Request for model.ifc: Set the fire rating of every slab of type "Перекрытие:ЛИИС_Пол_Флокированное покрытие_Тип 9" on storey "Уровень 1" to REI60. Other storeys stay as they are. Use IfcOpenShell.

First a look at what the model holds.

```python
import ifcopenshell
import ifcopenshell.util.element

model = ifcopenshell.open("model.ifc")
print(model.schema)
storey = next(s for s in model.by_type("IfcBuildingStorey") if s.Name == "Уровень 1")
slabs = [e for e in ifcopenshell.util.element.get_decomposition(storey) if e.is_a("IfcSlab")]
seen = {}
for e in slabs:
    element_type = ifcopenshell.util.element.get_type(e)
    key = (element_type.Name if element_type != e and element_type else None, ifcopenshell.util.element.get_pset(e, "Pset_SlabCommon", "FireRating"))
    seen[key] = seen.get(key, 0) + 1
for (name, value), count in sorted(seen.items(), key=str):
    print(count, "x", name, "|", value)
```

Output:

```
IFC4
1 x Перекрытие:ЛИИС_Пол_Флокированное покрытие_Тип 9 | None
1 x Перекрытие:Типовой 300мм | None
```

```python
import ifcopenshell
import ifcopenshell.api.pset
import ifcopenshell.util.element

model = ifcopenshell.open("model.ifc")

storey = next(s for s in model.by_type("IfcBuildingStorey") if s.Name == "Уровень 1")
slabs = [e for e in ifcopenshell.util.element.get_decomposition(storey) if e.is_a("IfcSlab")]

count = 0
for e in slabs:
    element_type = ifcopenshell.util.element.get_type(e)
    if element_type in (None, e) or element_type.Name != "Перекрытие:ЛИИС_Пол_Флокированное покрытие_Тип 9":
        continue
    # add_pset returns the element's existing set when there is one.
    pset = ifcopenshell.api.pset.add_pset(model, product=e, name="Pset_SlabCommon")
    ifcopenshell.api.pset.edit_pset(model, pset=pset, properties={"FireRating": "REI60"})
    count += 1

print(count, "slabs updated")

model.write("model_rev.ifc")
```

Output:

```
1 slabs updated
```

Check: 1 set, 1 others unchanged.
